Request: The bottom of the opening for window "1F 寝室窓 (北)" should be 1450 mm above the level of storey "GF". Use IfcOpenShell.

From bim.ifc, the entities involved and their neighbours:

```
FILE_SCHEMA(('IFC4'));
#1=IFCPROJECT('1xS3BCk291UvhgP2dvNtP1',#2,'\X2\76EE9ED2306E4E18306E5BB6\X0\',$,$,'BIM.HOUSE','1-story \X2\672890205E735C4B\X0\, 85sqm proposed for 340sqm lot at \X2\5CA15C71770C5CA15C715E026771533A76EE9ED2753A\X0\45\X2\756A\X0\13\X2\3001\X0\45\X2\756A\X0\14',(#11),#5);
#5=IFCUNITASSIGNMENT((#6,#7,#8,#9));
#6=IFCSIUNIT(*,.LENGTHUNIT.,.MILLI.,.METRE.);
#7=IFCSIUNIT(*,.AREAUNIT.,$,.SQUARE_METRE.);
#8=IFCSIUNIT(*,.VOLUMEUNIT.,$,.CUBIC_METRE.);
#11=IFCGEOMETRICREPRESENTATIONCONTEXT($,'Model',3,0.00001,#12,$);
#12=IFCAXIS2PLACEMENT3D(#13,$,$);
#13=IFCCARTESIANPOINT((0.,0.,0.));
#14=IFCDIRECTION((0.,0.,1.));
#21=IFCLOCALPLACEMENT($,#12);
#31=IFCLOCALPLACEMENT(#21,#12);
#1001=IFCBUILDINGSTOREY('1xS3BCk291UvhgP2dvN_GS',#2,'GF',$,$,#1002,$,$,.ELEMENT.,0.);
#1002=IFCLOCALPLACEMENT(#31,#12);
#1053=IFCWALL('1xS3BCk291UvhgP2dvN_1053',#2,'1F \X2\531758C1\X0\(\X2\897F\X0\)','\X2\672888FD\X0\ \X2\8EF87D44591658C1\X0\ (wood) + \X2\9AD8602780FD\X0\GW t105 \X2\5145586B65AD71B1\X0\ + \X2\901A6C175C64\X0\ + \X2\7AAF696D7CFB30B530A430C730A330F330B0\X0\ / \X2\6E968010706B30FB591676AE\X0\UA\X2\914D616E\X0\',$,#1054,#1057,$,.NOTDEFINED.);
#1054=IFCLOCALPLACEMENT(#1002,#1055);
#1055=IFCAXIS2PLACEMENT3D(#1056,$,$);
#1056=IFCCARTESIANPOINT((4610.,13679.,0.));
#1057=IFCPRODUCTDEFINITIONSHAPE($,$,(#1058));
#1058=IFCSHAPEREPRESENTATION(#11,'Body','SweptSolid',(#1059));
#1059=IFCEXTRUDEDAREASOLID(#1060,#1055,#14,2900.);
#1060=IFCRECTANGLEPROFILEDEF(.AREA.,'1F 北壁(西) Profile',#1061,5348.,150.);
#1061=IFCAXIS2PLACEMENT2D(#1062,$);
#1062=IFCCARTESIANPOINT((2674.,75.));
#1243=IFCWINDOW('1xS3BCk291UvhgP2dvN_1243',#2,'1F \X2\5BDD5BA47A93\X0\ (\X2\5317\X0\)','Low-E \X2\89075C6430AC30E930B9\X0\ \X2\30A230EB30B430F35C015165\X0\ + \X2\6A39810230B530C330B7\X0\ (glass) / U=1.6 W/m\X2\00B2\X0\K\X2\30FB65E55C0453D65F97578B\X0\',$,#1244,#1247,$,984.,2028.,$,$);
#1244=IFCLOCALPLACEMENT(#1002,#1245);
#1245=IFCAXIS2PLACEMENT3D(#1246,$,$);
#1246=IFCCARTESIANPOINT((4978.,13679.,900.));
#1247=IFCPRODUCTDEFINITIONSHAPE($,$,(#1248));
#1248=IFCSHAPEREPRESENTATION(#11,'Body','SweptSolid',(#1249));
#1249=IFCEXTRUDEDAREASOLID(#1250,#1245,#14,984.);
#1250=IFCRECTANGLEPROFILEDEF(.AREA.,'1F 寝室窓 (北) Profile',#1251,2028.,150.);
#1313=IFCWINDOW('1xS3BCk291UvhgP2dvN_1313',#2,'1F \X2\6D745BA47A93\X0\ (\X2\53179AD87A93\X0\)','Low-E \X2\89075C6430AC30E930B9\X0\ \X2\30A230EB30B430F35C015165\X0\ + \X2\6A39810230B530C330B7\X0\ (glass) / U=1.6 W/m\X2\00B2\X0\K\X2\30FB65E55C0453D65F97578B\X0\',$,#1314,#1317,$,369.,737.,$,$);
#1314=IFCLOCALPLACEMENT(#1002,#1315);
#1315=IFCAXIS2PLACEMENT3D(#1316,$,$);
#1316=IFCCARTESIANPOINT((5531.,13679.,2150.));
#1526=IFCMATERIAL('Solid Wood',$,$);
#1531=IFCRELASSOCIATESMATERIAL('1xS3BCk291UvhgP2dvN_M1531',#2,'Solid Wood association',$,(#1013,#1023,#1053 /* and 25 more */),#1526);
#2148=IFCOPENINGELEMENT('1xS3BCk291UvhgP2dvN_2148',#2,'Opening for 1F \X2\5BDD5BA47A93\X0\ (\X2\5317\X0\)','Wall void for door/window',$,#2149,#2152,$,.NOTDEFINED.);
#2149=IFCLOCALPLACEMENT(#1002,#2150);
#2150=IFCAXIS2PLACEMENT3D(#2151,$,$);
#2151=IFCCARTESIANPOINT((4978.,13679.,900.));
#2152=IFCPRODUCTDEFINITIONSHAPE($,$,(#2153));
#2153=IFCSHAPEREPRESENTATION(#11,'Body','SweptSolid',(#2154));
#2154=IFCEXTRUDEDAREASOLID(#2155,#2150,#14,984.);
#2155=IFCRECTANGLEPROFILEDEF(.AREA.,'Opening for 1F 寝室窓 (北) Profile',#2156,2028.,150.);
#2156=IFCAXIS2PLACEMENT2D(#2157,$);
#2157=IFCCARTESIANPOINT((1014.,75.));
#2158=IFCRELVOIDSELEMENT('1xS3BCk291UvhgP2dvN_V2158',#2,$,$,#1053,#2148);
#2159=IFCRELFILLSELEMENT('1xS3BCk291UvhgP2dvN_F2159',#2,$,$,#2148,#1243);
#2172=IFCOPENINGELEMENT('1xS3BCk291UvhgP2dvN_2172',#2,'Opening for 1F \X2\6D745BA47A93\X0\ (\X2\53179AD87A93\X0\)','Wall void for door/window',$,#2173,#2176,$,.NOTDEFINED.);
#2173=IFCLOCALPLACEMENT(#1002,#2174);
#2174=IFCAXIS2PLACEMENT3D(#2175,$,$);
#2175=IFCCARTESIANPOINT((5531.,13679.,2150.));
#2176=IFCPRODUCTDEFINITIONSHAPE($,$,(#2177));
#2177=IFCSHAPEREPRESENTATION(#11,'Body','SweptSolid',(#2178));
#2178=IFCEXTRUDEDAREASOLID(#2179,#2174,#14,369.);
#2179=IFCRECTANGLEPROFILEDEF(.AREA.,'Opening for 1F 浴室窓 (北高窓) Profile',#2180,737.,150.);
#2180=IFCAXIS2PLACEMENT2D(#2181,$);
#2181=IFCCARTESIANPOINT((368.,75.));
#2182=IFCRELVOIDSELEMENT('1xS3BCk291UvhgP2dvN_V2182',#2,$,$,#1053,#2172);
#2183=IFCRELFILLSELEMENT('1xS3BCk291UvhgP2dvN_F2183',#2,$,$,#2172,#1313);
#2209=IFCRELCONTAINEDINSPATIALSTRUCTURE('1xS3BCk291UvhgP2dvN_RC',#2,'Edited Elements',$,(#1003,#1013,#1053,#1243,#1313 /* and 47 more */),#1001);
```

```python
import numpy as np
import ifcopenshell
import ifcopenshell.api.geometry
import ifcopenshell.geom
import ifcopenshell.util.element
import ifcopenshell.util.placement
import ifcopenshell.util.shape
import ifcopenshell.util.unit

model = ifcopenshell.open("bim.ifc")
unit_scale = ifcopenshell.util.unit.calculate_unit_scale(model)

window = model.by_guid("1xS3BCk291UvhgP2dvN_1243")
opening = window.FillsVoids[0].RelatingOpeningElement
storey = ifcopenshell.util.element.get_container(window, ifc_class="IfcBuildingStorey")
level = ifcopenshell.util.placement.get_local_placement(storey.ObjectPlacement)[2, 3]

# The opening's origin need not be at the sill, so measure its lowest point.
shape = ifcopenshell.geom.create_shape(ifcopenshell.geom.settings(), opening)
bottom = ifcopenshell.util.shape.get_shape_bottom_elevation(shape, shape.geometry) / unit_scale
dz = level + 1.45 / unit_scale - bottom

shift = np.array([0.0, 0.0, dz])
# The window is not placed relative to its opening, so move both.
for product in (opening, window):
    matrix = ifcopenshell.util.placement.get_local_placement(product.ObjectPlacement)
    matrix[:3, 3] += shift
    ifcopenshell.api.geometry.edit_object_placement(model, product=product, matrix=matrix, is_si=False)

print(f"moved by {dz * unit_scale:+.3f} m")

model.write("bim-out.ifc")
```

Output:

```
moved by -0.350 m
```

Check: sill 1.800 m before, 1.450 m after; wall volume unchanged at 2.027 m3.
